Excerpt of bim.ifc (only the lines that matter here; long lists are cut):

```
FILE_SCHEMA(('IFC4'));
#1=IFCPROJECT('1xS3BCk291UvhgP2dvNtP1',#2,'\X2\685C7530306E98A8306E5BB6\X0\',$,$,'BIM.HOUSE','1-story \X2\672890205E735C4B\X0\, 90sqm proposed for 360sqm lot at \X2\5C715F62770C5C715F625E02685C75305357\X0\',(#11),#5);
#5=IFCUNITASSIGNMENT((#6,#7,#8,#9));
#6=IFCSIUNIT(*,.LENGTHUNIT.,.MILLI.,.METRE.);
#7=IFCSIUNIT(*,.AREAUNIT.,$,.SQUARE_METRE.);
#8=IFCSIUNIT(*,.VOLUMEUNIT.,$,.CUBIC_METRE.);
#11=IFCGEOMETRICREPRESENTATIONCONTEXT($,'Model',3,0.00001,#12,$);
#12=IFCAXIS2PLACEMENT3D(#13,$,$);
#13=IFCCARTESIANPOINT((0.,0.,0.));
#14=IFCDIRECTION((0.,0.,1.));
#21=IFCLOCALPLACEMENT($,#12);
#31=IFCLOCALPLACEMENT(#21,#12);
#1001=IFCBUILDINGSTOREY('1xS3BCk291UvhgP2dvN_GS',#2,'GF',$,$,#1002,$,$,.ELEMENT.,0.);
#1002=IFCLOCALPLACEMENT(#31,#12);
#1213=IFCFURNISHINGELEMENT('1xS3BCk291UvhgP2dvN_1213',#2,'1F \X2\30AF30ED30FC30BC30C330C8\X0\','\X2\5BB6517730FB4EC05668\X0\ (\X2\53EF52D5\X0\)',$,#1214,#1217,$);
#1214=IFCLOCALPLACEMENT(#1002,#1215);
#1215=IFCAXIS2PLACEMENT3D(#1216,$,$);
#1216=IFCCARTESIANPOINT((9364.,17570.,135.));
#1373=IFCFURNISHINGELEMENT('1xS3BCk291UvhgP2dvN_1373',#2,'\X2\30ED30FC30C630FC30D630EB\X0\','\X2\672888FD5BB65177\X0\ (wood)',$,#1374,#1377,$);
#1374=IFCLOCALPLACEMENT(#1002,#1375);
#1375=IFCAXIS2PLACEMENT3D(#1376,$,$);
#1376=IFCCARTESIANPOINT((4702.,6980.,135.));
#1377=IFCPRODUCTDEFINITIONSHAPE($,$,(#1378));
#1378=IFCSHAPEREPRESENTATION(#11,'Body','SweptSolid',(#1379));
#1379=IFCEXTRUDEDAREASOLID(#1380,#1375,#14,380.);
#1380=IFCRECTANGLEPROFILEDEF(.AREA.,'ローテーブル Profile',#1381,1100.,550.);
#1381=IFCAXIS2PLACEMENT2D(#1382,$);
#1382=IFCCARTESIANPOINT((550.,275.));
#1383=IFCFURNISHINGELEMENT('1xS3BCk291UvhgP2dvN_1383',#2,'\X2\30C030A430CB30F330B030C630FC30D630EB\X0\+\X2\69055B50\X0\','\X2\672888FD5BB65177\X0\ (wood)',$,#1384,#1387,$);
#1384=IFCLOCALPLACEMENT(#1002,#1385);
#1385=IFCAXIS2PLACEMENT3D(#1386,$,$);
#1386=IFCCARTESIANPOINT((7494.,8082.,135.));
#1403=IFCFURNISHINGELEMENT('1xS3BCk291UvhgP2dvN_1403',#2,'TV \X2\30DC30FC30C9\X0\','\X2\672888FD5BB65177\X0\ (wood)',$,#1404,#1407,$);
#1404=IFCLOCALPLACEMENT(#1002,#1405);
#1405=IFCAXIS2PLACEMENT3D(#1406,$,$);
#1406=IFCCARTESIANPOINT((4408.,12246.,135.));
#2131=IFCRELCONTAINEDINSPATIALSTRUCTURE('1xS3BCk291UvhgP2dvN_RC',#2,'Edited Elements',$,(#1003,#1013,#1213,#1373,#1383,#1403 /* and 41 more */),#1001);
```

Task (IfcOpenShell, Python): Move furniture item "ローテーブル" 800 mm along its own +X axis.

```python
import ifcopenshell
import ifcopenshell.api.geometry
import ifcopenshell.util.placement

model = ifcopenshell.open("bim.ifc")

item = model.by_guid("1xS3BCk291UvhgP2dvN_1373")
matrix = ifcopenshell.util.placement.get_local_placement(item.ObjectPlacement)
matrix[:3, 3] += matrix[:3, 0] * 800.0
ifcopenshell.api.geometry.edit_object_placement(model, product=item, matrix=matrix, is_si=False)

print(ifcopenshell.util.placement.get_local_placement(item.ObjectPlacement).round(3) + 0.0)

model.write("bim_v2.ifc")
```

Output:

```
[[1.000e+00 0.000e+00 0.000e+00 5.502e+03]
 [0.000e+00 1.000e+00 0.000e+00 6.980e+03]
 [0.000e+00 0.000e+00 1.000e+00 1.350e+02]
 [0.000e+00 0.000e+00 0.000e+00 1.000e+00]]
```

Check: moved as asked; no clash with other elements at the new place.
